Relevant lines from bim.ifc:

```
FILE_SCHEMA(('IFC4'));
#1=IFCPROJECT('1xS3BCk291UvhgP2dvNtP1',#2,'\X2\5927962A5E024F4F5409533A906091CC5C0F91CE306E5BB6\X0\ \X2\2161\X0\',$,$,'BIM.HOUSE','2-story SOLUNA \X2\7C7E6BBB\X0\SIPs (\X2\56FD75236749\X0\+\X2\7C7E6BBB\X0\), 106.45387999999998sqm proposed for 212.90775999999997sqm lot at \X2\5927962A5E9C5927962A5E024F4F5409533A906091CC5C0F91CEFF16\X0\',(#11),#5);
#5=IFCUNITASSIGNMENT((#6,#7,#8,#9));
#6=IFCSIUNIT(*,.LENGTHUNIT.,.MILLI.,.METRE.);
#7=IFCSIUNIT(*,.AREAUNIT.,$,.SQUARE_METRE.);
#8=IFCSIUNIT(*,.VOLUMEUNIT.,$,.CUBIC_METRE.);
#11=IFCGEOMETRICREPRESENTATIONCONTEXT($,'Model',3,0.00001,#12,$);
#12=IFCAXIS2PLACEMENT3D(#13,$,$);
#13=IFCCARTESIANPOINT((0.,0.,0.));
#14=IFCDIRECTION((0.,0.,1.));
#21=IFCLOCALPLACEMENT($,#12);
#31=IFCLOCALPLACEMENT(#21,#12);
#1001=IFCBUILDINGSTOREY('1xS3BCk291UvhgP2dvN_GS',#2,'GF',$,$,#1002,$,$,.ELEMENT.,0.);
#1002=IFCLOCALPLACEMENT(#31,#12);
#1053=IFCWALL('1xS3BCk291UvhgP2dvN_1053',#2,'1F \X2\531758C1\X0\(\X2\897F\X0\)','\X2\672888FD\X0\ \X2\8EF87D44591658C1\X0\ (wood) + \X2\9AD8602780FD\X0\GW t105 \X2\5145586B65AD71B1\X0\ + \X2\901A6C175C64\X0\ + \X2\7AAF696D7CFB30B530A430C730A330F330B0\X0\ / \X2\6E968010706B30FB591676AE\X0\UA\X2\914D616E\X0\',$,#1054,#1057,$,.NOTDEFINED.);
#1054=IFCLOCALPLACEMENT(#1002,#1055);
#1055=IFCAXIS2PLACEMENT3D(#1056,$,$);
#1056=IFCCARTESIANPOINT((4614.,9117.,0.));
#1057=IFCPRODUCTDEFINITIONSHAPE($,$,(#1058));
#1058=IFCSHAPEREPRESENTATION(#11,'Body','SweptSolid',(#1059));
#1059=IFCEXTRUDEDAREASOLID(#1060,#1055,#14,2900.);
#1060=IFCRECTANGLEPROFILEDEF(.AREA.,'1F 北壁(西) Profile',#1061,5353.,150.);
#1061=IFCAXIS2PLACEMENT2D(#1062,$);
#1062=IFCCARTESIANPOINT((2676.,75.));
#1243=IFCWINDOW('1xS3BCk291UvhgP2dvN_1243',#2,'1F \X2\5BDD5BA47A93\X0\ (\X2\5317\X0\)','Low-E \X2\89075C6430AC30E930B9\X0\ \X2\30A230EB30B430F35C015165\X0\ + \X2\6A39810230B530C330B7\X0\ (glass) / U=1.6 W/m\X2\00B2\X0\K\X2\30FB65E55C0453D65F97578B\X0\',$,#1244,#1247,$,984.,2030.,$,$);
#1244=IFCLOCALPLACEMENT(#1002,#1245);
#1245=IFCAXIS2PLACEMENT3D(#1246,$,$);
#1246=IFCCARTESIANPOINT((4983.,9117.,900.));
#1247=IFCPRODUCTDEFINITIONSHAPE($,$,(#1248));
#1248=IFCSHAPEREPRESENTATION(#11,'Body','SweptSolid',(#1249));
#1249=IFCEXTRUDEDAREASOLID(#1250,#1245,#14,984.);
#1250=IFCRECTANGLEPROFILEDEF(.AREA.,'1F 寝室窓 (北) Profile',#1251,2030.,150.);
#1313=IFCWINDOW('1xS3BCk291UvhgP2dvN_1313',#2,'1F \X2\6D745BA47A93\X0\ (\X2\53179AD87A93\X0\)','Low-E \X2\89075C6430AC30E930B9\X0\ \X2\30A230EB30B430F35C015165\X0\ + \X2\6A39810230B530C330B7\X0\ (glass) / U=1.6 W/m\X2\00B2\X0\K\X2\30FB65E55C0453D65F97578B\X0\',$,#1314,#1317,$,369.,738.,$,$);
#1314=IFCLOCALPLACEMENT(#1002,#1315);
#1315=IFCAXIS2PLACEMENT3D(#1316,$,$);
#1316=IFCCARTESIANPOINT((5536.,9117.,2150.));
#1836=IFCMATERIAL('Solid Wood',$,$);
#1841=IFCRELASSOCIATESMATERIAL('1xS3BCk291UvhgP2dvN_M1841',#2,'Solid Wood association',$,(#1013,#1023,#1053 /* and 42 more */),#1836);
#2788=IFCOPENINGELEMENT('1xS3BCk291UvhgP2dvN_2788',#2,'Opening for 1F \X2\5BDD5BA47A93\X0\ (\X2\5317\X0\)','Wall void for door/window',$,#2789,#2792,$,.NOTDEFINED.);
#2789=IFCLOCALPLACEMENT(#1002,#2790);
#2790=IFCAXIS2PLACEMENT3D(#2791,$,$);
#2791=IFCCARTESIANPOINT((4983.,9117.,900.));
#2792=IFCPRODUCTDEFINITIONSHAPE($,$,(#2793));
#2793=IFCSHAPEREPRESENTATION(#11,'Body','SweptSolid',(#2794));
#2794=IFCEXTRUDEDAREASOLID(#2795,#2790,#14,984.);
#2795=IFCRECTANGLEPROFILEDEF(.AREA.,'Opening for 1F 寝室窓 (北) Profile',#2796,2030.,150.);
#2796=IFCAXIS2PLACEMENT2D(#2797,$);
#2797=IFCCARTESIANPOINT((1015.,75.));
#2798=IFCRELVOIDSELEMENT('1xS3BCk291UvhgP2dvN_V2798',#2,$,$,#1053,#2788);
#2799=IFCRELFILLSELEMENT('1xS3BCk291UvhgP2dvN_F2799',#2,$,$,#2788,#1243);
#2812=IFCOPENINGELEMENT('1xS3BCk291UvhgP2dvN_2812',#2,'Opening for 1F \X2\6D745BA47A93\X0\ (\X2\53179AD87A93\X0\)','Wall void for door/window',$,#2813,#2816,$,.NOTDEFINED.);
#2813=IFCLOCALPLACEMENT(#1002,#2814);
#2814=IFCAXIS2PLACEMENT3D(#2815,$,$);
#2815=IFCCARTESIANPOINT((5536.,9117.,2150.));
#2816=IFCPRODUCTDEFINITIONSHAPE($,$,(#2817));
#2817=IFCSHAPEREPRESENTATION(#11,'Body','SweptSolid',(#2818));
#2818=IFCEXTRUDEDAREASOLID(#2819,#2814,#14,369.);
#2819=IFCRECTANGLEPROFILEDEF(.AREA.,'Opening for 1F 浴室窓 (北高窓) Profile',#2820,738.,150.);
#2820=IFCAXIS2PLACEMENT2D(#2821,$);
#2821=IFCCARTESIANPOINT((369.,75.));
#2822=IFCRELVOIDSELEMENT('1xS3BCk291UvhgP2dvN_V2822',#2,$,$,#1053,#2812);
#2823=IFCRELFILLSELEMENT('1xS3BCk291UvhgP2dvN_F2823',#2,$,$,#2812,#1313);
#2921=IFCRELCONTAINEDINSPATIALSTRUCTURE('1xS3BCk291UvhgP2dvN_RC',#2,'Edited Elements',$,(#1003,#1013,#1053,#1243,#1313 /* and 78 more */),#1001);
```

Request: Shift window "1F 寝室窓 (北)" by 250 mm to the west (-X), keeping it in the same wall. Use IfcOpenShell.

```python
import ifcopenshell
import ifcopenshell.api.geometry
import ifcopenshell.util.placement

model = ifcopenshell.open("bim.ifc")

window = model.by_guid("1xS3BCk291UvhgP2dvN_1243")
opening = window.FillsVoids[0].RelatingOpeningElement
wall = opening.VoidsElements[0].RelatingBuildingElement

wall_matrix = ifcopenshell.util.placement.get_local_placement(wall.ObjectPlacement)
shift = wall_matrix[:3, 0] * -250.0
before = ifcopenshell.util.placement.get_local_placement(window.ObjectPlacement)[:3, 3].copy()

# The window is not placed relative to its opening, so move both.
for product in (opening, window):
    matrix = ifcopenshell.util.placement.get_local_placement(product.ObjectPlacement)
    matrix[:3, 3] += shift
    ifcopenshell.api.geometry.edit_object_placement(model, product=product, matrix=matrix, is_si=False)

after = ifcopenshell.util.placement.get_local_placement(window.ObjectPlacement)[:3, 3]
print("window moved by", (after - before).round(3) + 0.0)

model.write("bim-out.ifc")
```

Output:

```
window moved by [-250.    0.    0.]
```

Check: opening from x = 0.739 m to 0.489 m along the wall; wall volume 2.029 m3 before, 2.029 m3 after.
